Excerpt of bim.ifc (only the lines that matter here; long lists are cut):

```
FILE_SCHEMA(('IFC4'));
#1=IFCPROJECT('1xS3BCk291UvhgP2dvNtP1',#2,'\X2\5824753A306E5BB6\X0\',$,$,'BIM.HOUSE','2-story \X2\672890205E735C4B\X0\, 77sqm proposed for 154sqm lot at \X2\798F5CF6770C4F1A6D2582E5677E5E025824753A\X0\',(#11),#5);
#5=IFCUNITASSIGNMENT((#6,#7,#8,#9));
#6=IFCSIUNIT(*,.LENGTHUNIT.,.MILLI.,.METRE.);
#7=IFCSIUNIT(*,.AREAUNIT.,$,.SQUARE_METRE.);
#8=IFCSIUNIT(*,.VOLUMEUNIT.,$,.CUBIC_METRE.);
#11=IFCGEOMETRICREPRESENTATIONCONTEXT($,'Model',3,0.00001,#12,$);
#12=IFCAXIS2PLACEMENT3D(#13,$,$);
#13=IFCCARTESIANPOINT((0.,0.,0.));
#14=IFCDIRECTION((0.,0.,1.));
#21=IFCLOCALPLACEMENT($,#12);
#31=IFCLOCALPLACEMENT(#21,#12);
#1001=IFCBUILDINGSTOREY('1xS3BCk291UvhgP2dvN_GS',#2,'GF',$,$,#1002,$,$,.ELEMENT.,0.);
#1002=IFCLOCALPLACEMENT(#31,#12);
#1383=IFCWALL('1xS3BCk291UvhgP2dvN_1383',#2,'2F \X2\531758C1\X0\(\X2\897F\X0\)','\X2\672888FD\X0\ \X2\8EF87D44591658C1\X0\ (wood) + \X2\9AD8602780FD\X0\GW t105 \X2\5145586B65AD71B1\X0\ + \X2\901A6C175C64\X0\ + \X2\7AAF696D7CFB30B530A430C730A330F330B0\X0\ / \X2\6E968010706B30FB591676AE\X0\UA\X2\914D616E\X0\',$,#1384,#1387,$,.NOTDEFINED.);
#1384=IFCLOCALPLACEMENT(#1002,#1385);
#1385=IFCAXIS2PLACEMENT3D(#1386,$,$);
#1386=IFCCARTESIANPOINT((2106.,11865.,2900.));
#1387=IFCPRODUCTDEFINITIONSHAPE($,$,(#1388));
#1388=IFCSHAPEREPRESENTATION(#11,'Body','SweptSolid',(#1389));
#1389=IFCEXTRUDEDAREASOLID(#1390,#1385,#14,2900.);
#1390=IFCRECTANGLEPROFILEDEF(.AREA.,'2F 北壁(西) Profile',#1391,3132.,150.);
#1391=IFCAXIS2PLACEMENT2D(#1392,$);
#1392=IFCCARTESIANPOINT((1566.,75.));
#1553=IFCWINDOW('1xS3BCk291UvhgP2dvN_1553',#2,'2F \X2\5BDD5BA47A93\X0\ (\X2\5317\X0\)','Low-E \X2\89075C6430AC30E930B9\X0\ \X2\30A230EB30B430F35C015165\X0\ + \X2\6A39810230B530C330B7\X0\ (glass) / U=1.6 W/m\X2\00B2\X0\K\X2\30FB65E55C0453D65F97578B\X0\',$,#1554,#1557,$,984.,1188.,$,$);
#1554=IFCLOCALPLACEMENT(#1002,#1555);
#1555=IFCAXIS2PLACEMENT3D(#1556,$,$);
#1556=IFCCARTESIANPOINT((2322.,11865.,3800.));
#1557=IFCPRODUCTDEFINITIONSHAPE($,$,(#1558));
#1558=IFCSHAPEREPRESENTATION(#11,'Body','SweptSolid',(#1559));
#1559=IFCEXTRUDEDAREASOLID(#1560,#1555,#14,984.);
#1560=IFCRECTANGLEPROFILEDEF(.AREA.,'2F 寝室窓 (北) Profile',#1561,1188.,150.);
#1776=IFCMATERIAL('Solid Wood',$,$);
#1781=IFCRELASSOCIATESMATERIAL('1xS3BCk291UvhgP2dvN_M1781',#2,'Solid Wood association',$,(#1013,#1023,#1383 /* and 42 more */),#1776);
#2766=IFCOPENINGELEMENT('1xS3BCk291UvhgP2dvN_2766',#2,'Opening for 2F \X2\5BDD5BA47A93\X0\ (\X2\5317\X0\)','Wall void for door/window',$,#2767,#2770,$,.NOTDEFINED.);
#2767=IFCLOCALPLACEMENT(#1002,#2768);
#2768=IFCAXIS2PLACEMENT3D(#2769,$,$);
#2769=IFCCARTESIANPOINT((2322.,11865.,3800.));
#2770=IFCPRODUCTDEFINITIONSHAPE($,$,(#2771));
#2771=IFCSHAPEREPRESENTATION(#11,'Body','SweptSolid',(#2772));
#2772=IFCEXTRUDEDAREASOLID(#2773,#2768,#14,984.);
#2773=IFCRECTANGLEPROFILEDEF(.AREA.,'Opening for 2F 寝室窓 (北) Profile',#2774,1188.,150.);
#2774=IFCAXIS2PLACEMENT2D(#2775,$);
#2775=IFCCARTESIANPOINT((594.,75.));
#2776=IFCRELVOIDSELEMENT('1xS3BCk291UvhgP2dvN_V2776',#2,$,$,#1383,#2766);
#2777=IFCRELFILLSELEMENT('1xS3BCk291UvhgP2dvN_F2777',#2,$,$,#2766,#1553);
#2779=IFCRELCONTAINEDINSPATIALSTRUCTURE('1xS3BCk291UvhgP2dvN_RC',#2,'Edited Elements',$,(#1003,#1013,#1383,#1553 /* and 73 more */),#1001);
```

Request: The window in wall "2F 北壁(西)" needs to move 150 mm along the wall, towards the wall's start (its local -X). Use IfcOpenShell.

```python
import ifcopenshell
import ifcopenshell.api.geometry
import ifcopenshell.util.placement

model = ifcopenshell.open("bim.ifc")

window = model.by_guid("1xS3BCk291UvhgP2dvN_1553")
opening = window.FillsVoids[0].RelatingOpeningElement
wall = opening.VoidsElements[0].RelatingBuildingElement

wall_matrix = ifcopenshell.util.placement.get_local_placement(wall.ObjectPlacement)
shift = wall_matrix[:3, 0] * -150.0
before = ifcopenshell.util.placement.get_local_placement(window.ObjectPlacement)[:3, 3].copy()

# The window is not placed relative to its opening, so move both.
for product in (opening, window):
    matrix = ifcopenshell.util.placement.get_local_placement(product.ObjectPlacement)
    matrix[:3, 3] += shift
    ifcopenshell.api.geometry.edit_object_placement(model, product=product, matrix=matrix, is_si=False)

after = ifcopenshell.util.placement.get_local_placement(window.ObjectPlacement)[:3, 3]
print("window moved by", (after - before).round(3) + 0.0)

model.write("bim-out.ifc")
```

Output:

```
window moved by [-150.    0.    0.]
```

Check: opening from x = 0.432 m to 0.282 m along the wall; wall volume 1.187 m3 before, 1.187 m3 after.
